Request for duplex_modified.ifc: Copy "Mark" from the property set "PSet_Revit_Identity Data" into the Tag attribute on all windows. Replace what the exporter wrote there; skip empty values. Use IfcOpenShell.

First a look at what the model holds.

```python
import ifcopenshell
import ifcopenshell.util.element

model = ifcopenshell.open("duplex_modified.ifc")
print(model.schema)
windows = model.by_type("IfcWindow")
print(len(windows), "windows")
for e in windows[:8]:
    source = ifcopenshell.util.element.get_pset(e, "PSet_Revit_Identity Data", "Mark")
    target = e.Tag
    print(e.id(), repr(source), repr(target), sep=" | ")
```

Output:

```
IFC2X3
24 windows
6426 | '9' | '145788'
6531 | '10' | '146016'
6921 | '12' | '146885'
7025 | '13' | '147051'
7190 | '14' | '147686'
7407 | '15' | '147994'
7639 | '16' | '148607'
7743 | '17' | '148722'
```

```python
import ifcopenshell
import ifcopenshell.util.element

model = ifcopenshell.open("duplex_modified.ifc")

count = 0
for e in model.by_type("IfcWindow"):
    value = ifcopenshell.util.element.get_pset(e, "PSet_Revit_Identity Data", "Mark")
    current = e.Tag
    if not value or not value.strip() or current == value:
        continue
    e.Tag = value
    count += 1

print(count, "windows updated")

model.write("duplex_modified_rev.ifc")
```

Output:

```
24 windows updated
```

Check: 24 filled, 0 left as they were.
